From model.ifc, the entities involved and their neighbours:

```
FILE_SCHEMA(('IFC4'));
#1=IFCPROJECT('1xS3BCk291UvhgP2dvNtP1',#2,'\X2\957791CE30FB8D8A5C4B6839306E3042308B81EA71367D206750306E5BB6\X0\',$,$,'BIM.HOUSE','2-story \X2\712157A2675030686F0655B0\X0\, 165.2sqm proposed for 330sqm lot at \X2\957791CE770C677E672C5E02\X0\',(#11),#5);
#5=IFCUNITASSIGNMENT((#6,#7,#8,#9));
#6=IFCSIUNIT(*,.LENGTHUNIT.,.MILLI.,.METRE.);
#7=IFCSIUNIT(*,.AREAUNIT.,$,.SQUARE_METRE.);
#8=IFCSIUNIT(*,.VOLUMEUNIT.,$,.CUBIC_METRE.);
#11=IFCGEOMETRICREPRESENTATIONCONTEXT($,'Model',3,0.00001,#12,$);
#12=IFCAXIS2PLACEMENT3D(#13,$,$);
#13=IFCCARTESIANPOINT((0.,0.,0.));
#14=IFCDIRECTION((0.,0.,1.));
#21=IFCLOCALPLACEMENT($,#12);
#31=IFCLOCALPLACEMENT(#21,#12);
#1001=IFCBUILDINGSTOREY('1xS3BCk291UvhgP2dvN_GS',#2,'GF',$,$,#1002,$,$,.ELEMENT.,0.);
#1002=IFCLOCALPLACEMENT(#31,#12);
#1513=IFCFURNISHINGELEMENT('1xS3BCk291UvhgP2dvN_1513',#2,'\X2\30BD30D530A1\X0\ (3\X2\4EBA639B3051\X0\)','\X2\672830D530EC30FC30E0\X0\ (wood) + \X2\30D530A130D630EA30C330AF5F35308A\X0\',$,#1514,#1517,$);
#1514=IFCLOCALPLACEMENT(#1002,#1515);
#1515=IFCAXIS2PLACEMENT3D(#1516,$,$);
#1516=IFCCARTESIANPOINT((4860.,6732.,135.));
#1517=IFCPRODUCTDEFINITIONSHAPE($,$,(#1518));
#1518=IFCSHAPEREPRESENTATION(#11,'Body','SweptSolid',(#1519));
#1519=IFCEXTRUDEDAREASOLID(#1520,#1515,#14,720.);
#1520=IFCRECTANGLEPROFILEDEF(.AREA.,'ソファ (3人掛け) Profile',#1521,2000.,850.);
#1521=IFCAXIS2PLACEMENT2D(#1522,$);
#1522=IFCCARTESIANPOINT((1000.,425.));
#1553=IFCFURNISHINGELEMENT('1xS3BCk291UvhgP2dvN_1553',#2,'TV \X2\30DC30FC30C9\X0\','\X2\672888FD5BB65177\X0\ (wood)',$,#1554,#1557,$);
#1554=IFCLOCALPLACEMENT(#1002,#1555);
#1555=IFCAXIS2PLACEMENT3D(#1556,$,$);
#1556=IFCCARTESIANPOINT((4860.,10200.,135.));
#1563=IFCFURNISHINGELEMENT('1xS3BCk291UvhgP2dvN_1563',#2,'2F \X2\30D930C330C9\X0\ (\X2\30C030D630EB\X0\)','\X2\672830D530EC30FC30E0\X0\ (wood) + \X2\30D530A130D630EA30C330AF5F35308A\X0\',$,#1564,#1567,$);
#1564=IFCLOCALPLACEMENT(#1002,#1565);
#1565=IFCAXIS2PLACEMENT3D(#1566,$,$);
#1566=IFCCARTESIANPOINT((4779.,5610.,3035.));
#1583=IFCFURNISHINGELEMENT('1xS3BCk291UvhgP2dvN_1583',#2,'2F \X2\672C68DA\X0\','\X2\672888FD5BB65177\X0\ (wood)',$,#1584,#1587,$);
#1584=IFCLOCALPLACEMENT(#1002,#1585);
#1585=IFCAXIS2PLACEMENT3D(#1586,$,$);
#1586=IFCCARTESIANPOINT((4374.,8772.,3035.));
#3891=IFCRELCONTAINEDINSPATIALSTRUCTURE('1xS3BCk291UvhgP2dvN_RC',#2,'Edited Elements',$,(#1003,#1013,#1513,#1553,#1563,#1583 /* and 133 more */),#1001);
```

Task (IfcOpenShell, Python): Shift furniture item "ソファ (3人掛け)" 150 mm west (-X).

```python
import ifcopenshell
import ifcopenshell.api.geometry
import ifcopenshell.util.placement
import ifcopenshell.util.unit

model = ifcopenshell.open("model.ifc")
unit_scale = ifcopenshell.util.unit.calculate_unit_scale(model)

item = model.by_guid("1xS3BCk291UvhgP2dvN_1513")
matrix = ifcopenshell.util.placement.get_local_placement(item.ObjectPlacement)
matrix[0, 3] -= 0.15 / unit_scale
ifcopenshell.api.geometry.edit_object_placement(model, product=item, matrix=matrix, is_si=False)

print(ifcopenshell.util.placement.get_local_placement(item.ObjectPlacement).round(3) + 0.0)

model.write("model_updated.ifc")
```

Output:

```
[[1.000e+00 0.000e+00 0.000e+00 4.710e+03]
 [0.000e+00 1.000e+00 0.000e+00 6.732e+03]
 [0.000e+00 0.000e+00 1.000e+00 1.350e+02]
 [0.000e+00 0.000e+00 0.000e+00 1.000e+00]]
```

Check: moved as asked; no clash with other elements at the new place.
